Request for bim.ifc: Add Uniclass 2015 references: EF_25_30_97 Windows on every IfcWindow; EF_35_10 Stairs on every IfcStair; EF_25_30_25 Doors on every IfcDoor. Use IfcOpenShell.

First a look at what the model holds.

```python
import ifcopenshell

model = ifcopenshell.open("bim.ifc")
print(model.schema)
print("classifications:", [c.Name for c in model.by_type("IfcClassification")])
for ifc_class in ("IfcDoor", "IfcRoof", "IfcStair", "IfcWall", "IfcWindow"):
    print(ifc_class, len(model.by_type(ifc_class)))
```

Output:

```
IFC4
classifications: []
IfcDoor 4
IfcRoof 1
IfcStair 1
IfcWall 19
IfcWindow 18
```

```python
import ifcopenshell
import ifcopenshell.api.classification

model = ifcopenshell.open("bim.ifc")

system = ifcopenshell.api.classification.add_classification(model, classification="Uniclass 2015")

codes = {
    "IfcWindow": ("EF_25_30_97", "Windows"),
    "IfcStair": ("EF_35_10", "Stairs"),
    "IfcDoor": ("EF_25_30_25", "Doors"),
}
for ifc_class, (code, name) in codes.items():
    products = model.by_type(ifc_class)
    ifcopenshell.api.classification.add_reference(
        model, products=products, classification=system, identification=code, name=name
    )
    print(code, len(products))

model.write("bim_v2.ifc")
```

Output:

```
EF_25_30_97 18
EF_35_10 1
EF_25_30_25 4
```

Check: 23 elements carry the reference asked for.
